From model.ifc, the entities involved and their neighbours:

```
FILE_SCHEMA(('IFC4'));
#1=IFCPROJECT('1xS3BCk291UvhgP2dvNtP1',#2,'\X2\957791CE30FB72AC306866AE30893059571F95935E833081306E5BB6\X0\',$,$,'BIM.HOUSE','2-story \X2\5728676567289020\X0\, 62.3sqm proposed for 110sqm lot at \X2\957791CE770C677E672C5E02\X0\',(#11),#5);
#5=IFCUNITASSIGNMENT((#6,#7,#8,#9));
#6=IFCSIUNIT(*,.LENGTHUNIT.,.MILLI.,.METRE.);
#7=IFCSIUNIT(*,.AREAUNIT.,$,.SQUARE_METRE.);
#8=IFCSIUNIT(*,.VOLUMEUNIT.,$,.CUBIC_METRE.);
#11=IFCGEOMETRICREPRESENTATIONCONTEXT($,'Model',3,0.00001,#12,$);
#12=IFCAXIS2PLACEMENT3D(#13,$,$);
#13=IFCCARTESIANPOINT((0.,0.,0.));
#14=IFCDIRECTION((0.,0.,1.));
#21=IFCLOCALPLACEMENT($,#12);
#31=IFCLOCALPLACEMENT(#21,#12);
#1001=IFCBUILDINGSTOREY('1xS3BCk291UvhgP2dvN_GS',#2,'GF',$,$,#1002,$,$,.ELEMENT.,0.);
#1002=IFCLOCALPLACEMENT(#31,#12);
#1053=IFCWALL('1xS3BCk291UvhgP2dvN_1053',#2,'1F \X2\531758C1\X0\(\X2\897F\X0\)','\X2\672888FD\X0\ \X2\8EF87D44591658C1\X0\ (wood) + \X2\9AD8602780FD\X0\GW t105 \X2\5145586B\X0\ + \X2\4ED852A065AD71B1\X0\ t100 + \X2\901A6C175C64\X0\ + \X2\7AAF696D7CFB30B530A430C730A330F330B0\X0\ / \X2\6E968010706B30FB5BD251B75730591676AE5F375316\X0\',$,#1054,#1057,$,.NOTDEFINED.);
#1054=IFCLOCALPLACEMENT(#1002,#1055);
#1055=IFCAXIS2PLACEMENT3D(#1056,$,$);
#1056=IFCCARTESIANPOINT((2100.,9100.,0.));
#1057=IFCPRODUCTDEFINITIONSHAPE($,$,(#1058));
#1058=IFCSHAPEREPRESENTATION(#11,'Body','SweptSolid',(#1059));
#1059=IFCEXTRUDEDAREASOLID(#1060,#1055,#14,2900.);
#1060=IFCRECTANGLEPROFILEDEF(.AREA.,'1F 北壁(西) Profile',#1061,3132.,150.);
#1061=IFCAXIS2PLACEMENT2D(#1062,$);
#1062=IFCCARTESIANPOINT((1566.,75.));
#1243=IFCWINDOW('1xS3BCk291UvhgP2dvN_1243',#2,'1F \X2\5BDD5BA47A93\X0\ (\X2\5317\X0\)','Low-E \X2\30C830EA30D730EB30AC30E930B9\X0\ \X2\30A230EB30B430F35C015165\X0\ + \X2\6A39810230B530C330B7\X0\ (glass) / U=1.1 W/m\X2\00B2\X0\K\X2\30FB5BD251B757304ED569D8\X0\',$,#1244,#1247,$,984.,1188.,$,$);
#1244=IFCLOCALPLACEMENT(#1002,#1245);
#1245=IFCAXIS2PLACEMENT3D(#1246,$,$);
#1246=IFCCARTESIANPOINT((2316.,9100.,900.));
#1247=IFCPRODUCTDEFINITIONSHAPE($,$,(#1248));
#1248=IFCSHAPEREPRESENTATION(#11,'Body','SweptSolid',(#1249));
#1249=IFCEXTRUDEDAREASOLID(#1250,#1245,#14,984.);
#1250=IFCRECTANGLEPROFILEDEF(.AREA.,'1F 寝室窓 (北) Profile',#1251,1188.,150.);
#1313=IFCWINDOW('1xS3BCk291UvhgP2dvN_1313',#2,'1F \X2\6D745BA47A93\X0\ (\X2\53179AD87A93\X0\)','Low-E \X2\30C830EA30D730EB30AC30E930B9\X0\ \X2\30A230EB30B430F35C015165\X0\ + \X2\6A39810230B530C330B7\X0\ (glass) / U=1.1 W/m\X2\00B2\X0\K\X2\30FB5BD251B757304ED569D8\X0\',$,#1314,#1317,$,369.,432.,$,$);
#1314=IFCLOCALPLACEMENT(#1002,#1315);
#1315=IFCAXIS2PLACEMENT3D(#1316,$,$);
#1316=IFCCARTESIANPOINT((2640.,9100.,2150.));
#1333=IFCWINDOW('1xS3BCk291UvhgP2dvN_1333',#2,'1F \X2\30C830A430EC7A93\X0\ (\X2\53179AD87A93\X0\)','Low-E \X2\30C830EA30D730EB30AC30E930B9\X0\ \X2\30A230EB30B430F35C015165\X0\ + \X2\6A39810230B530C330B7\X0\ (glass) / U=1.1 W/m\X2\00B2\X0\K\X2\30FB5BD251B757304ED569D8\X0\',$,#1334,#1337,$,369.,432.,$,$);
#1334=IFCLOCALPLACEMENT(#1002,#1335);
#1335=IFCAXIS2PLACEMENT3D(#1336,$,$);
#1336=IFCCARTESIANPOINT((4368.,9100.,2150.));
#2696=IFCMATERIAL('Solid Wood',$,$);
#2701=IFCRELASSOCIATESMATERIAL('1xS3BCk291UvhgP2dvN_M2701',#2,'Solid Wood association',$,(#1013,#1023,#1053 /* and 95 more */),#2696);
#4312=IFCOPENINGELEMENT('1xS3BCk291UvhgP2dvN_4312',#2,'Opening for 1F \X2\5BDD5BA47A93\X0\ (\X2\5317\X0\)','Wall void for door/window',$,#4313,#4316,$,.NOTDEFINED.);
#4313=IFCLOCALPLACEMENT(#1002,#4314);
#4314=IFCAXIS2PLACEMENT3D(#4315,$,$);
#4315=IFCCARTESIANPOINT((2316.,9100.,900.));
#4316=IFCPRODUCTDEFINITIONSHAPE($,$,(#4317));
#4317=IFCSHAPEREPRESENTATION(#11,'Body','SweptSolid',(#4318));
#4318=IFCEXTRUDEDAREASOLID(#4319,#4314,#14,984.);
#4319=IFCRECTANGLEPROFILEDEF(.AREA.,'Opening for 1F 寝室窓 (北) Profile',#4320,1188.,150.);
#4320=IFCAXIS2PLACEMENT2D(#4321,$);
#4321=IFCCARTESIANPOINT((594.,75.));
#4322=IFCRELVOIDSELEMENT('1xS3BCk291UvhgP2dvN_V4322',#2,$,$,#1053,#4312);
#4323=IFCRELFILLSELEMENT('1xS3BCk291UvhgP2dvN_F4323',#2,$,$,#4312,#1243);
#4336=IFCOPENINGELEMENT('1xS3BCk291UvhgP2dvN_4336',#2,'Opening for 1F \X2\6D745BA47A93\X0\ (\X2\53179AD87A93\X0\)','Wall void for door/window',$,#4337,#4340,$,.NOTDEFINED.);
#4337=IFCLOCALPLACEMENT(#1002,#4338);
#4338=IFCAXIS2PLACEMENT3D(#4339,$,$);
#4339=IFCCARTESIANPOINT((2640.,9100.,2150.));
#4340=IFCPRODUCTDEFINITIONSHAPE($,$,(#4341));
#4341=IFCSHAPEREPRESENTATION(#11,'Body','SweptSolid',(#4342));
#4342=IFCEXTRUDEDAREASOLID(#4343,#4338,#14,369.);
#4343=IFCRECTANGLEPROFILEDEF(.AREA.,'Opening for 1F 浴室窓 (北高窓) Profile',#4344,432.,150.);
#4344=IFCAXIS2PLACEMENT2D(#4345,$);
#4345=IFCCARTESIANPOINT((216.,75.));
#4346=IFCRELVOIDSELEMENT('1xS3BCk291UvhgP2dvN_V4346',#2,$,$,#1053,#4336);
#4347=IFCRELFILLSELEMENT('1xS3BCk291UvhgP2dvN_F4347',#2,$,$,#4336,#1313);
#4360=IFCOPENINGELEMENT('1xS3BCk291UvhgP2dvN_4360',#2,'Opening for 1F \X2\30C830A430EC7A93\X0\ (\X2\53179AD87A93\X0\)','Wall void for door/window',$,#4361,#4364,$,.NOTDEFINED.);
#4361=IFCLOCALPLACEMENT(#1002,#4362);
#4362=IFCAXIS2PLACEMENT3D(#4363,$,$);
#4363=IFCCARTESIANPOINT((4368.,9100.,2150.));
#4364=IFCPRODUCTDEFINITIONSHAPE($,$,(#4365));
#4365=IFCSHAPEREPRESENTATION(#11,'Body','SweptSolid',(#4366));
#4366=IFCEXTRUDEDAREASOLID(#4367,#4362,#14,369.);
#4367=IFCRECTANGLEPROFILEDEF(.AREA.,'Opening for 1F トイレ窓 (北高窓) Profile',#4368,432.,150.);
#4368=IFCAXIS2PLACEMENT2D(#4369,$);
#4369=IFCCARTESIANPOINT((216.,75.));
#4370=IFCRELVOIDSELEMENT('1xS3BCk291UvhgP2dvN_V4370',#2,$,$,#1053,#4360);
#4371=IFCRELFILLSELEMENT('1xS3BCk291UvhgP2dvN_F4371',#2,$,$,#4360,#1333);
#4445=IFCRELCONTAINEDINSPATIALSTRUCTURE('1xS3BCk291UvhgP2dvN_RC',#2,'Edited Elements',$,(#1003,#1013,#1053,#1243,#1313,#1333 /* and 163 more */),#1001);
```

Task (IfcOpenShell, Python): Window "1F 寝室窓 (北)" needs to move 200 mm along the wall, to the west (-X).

```python
import ifcopenshell
import ifcopenshell.api.geometry
import ifcopenshell.util.placement
import ifcopenshell.util.unit

model = ifcopenshell.open("model.ifc")
unit_scale = ifcopenshell.util.unit.calculate_unit_scale(model)

window = model.by_guid("1xS3BCk291UvhgP2dvN_1243")
opening = window.FillsVoids[0].RelatingOpeningElement
wall = opening.VoidsElements[0].RelatingBuildingElement

wall_matrix = ifcopenshell.util.placement.get_local_placement(wall.ObjectPlacement)
shift = wall_matrix[:3, 0] * -0.2 / unit_scale
before = ifcopenshell.util.placement.get_local_placement(window.ObjectPlacement)[:3, 3].copy()

# The window is not placed relative to its opening, so move both.
for product in (opening, window):
    matrix = ifcopenshell.util.placement.get_local_placement(product.ObjectPlacement)
    matrix[:3, 3] += shift
    ifcopenshell.api.geometry.edit_object_placement(model, product=product, matrix=matrix, is_si=False)

after = ifcopenshell.util.placement.get_local_placement(window.ObjectPlacement)[:3, 3]
print("window moved by", (after - before).round(3) + 0.0)

model.write("model_edited.ifc")
```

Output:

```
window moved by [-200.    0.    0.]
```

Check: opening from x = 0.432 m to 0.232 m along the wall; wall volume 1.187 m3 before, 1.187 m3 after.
